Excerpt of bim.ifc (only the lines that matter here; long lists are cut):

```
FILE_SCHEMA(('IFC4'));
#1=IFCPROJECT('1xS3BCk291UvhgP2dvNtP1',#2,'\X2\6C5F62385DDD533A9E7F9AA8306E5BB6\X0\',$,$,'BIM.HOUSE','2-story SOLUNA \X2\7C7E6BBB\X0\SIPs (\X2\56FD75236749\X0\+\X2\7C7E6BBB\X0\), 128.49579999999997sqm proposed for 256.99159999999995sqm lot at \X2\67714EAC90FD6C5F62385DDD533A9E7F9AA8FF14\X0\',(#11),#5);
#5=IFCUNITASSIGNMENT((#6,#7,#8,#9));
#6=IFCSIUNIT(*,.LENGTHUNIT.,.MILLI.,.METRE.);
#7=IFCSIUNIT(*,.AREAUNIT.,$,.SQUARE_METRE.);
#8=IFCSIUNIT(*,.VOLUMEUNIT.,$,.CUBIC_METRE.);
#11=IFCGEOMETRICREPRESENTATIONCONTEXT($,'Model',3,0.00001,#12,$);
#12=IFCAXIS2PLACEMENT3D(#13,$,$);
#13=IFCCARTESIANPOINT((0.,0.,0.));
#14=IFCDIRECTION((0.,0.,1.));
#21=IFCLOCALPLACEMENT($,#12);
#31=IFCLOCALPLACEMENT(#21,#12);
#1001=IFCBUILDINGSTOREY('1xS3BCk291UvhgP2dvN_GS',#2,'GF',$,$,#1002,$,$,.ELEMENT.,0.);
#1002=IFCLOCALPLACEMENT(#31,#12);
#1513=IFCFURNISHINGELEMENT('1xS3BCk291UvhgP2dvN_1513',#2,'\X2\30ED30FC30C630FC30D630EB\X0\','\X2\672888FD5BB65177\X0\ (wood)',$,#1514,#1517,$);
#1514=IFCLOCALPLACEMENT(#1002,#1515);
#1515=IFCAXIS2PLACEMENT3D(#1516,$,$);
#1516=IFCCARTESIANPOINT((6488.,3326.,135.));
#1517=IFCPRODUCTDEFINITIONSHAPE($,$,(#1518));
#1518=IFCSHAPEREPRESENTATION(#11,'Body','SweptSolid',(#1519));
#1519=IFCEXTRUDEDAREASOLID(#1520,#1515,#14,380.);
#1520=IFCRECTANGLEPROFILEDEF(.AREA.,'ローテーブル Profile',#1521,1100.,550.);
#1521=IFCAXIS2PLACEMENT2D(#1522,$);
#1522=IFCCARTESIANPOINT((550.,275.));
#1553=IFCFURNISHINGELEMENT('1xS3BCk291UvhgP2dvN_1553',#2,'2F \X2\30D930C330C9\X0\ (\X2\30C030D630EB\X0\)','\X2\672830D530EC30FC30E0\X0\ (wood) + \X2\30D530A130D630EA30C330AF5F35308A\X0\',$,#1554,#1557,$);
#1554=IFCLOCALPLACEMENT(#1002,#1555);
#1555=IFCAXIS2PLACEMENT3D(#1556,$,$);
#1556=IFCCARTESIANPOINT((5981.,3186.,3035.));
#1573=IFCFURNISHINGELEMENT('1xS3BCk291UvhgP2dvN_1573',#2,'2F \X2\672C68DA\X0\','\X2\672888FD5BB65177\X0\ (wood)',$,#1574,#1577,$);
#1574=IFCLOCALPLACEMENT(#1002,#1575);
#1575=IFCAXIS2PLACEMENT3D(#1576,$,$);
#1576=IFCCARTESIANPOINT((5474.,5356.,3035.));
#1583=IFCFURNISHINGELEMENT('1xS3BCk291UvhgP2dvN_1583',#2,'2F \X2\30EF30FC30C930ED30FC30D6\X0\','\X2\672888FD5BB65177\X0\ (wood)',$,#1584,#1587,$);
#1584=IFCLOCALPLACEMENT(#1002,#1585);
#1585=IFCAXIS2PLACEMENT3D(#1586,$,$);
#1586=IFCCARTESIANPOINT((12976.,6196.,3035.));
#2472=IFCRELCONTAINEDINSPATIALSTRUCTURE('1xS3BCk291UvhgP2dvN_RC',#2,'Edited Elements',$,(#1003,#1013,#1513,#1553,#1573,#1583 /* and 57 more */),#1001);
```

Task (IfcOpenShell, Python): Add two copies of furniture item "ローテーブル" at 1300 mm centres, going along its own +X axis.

```python
import ifcopenshell
import ifcopenshell.api.geometry
import ifcopenshell.api.root
import ifcopenshell.util.element
import ifcopenshell.util.placement

model = ifcopenshell.open("bim.ifc")


def reuse_history(source, copy):
    """copy_class also copies each property set's owner history, people and application; keep the originals."""
    for rel in copy.IsDefinedBy:
        if rel.is_a("IfcRelDefinesByProperties") and (history := rel.RelatingPropertyDefinition.OwnerHistory):
            rel.RelatingPropertyDefinition.OwnerHistory = source.OwnerHistory
            ifcopenshell.util.element.remove_deep2(model, history)


source = model.by_guid("1xS3BCk291UvhgP2dvN_1513")
base = ifcopenshell.util.placement.get_local_placement(source.ObjectPlacement)
step = base[:3, 0] * 1300.0

for i in range(1, 3):
    copy = ifcopenshell.api.root.copy_class(model, product=source)
    copy.Representation = ifcopenshell.util.element.copy_deep(
        model, source.Representation, exclude=["IfcGeometricRepresentationContext", "IfcRepresentationMap"]
    )
    reuse_history(source, copy)
    matrix = base.copy()
    matrix[:3, 3] += i * step
    print("added at", matrix[:3, 3].round(3) + 0.0)
    ifcopenshell.api.geometry.edit_object_placement(model, product=copy, matrix=matrix, is_si=False)

model.write("bim_v2.ifc")
```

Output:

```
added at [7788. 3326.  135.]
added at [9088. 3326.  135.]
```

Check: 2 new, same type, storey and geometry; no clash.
